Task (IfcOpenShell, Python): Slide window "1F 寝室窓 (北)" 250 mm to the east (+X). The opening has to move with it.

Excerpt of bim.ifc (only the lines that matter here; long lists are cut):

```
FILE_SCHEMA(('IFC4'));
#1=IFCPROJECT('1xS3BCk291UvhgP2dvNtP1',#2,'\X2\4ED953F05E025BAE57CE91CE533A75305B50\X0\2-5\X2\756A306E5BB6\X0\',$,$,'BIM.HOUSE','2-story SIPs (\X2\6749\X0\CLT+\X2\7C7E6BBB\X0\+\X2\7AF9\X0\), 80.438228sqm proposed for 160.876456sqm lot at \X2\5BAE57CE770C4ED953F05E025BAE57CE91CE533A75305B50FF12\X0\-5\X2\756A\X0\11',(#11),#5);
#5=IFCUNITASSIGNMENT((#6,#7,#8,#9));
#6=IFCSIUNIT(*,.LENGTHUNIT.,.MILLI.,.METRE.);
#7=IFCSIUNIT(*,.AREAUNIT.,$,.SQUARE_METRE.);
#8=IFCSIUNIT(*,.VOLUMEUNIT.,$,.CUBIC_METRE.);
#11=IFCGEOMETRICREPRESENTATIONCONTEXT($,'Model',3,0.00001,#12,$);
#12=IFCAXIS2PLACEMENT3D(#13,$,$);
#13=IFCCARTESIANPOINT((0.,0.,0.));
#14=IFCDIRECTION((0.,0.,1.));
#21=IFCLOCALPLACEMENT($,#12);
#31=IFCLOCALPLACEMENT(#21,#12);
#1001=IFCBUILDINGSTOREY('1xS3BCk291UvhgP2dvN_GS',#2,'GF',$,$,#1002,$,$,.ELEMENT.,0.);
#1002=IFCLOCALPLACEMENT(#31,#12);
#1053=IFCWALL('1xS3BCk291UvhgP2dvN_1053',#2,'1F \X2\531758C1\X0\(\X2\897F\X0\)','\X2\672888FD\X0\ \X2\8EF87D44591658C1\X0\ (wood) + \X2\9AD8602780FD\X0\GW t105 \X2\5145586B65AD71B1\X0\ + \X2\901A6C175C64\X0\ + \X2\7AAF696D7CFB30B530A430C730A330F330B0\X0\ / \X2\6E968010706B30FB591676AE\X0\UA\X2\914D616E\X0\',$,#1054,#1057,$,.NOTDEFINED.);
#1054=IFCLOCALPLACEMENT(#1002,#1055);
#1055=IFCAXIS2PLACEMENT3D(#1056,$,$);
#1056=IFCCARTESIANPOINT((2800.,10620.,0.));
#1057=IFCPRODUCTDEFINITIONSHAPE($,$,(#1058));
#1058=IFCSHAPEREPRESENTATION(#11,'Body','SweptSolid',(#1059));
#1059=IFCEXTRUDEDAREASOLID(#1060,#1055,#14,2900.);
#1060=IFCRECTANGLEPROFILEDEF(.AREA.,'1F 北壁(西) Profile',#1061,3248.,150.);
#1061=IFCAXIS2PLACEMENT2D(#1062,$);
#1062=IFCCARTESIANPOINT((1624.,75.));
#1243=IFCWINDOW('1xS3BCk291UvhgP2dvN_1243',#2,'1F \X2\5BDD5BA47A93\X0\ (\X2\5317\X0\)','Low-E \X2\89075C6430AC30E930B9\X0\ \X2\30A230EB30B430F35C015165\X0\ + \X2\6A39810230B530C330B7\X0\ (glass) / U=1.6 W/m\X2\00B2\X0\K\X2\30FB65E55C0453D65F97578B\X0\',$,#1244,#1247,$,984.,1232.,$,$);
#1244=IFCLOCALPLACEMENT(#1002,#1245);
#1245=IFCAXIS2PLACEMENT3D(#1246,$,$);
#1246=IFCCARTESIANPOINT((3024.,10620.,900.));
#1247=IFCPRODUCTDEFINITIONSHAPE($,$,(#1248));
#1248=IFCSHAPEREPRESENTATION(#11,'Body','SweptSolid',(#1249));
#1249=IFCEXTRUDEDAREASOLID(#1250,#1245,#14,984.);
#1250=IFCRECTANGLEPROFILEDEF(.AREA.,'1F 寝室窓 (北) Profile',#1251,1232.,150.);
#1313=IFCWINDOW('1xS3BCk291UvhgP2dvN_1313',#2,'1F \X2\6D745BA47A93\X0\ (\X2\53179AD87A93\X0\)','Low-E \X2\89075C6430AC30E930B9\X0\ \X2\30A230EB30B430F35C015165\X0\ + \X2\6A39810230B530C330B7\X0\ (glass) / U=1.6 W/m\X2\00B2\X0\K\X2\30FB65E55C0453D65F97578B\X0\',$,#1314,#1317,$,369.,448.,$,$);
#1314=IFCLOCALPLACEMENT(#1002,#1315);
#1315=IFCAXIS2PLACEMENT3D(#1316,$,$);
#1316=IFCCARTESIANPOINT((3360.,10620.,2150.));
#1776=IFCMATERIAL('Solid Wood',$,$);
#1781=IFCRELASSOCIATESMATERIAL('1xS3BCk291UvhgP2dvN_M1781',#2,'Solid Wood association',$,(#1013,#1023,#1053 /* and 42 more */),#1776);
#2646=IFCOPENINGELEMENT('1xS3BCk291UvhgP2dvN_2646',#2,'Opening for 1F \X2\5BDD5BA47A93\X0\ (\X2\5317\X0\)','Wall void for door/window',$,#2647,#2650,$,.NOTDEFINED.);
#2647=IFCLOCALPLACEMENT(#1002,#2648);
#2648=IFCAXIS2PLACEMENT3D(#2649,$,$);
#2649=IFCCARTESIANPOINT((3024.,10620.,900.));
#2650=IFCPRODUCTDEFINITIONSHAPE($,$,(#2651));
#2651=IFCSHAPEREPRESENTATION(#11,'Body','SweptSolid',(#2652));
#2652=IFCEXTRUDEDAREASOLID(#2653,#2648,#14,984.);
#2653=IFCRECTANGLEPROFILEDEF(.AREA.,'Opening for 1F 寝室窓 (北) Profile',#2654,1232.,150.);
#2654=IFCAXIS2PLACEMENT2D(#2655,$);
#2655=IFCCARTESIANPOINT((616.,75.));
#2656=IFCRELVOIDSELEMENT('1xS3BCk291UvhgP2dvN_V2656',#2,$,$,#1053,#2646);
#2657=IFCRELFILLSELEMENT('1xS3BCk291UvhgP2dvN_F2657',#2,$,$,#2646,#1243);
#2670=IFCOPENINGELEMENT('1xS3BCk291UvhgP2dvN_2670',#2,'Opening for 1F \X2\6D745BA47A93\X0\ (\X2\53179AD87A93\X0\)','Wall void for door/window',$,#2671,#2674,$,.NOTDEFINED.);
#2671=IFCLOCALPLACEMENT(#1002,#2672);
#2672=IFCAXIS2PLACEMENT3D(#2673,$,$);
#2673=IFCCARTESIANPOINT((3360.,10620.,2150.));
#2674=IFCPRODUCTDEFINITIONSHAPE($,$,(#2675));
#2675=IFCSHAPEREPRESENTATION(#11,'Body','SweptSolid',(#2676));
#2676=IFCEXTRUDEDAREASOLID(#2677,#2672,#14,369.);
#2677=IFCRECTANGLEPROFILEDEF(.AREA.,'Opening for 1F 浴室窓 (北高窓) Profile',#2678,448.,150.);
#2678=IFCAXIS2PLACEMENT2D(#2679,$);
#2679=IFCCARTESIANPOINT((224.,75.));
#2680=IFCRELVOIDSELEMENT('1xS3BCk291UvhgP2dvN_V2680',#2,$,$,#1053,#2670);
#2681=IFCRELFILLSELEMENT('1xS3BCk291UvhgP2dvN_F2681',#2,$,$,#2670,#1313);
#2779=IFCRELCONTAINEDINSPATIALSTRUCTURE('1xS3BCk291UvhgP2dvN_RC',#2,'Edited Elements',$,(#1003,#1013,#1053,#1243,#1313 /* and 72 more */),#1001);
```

```python
import ifcopenshell
import ifcopenshell.api.geometry
import ifcopenshell.util.placement
import ifcopenshell.util.unit

model = ifcopenshell.open("bim.ifc")
unit_scale = ifcopenshell.util.unit.calculate_unit_scale(model)

window = model.by_guid("1xS3BCk291UvhgP2dvN_1243")
opening = window.FillsVoids[0].RelatingOpeningElement
wall = opening.VoidsElements[0].RelatingBuildingElement

wall_matrix = ifcopenshell.util.placement.get_local_placement(wall.ObjectPlacement)
shift = wall_matrix[:3, 0] * 0.25 / unit_scale
before = ifcopenshell.util.placement.get_local_placement(window.ObjectPlacement)[:3, 3].copy()

# The window is not placed relative to its opening, so move both.
for product in (opening, window):
    matrix = ifcopenshell.util.placement.get_local_placement(product.ObjectPlacement)
    matrix[:3, 3] += shift
    ifcopenshell.api.geometry.edit_object_placement(model, product=product, matrix=matrix, is_si=False)

after = ifcopenshell.util.placement.get_local_placement(window.ObjectPlacement)[:3, 3]
print("window moved by", (after - before).round(3) + 0.0)

model.write("bim_v2.ifc")
```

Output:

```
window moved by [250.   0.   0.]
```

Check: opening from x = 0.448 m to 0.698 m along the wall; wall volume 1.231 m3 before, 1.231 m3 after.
